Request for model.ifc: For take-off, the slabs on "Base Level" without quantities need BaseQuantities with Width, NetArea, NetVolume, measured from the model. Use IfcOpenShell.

First a look at what the model holds.

```python
import ifcopenshell
import ifcopenshell.util.element
import ifcopenshell.util.unit

model = ifcopenshell.open("model.ifc")
print(model.schema)
for unit_type in ("LENGTHUNIT", "AREAUNIT", "VOLUMEUNIT"):
    print(unit_type, ifcopenshell.util.unit.calculate_unit_scale(model, unit_type))
storey = next(s for s in model.by_type("IfcBuildingStorey") if s.Name == "Base Level")
slabs = [e for e in ifcopenshell.util.element.get_decomposition(storey) if e.is_a("IfcSlab")]
for e in sorted(slabs, key=lambda e: e.id()):
    print(e.id(), e.is_a(), e.Name, list(ifcopenshell.util.element.get_psets(e, qtos_only=True)), sep=" | ")
```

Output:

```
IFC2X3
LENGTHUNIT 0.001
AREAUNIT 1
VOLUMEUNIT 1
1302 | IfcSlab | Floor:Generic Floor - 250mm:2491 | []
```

```python
import ifcopenshell
import ifcopenshell.api.pset
import ifcopenshell.geom
import ifcopenshell.util.element
import ifcopenshell.util.shape
import ifcopenshell.util.unit

model = ifcopenshell.open("model.ifc")
unit_scale = ifcopenshell.util.unit.calculate_unit_scale(model)
area_scale = ifcopenshell.util.unit.calculate_unit_scale(model, "AREAUNIT")
volume_scale = ifcopenshell.util.unit.calculate_unit_scale(model, "VOLUMEUNIT")
settings = ifcopenshell.geom.settings()

storey = next(s for s in model.by_type("IfcBuildingStorey") if s.Name == "Base Level")
slabs = [e for e in ifcopenshell.util.element.get_decomposition(storey) if e.is_a("IfcSlab")]

for e in sorted(slabs, key=lambda e: e.id()):
    if ifcopenshell.util.element.get_psets(e, qtos_only=True, should_inherit=False):
        continue
    # Geometry comes back in metres, in the element's own axes.
    shape = ifcopenshell.geom.create_shape(settings, e)
    values = {
        "Width": ifcopenshell.util.shape.get_z(shape.geometry) / unit_scale,
        "NetArea": ifcopenshell.util.shape.get_footprint_area(shape.geometry) / area_scale,
        "NetVolume": ifcopenshell.util.shape.get_volume(shape.geometry) / volume_scale,
    }
    qto = ifcopenshell.api.pset.add_qto(model, product=e, name="BaseQuantities")
    ifcopenshell.api.pset.edit_qto(model, qto=qto, properties=values)
    print(e.id(), {k: round(v, 3) for k, v in values.items()})

model.write("model_rev.ifc")
```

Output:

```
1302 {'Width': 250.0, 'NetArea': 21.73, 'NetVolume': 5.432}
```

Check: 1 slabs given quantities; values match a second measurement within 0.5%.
